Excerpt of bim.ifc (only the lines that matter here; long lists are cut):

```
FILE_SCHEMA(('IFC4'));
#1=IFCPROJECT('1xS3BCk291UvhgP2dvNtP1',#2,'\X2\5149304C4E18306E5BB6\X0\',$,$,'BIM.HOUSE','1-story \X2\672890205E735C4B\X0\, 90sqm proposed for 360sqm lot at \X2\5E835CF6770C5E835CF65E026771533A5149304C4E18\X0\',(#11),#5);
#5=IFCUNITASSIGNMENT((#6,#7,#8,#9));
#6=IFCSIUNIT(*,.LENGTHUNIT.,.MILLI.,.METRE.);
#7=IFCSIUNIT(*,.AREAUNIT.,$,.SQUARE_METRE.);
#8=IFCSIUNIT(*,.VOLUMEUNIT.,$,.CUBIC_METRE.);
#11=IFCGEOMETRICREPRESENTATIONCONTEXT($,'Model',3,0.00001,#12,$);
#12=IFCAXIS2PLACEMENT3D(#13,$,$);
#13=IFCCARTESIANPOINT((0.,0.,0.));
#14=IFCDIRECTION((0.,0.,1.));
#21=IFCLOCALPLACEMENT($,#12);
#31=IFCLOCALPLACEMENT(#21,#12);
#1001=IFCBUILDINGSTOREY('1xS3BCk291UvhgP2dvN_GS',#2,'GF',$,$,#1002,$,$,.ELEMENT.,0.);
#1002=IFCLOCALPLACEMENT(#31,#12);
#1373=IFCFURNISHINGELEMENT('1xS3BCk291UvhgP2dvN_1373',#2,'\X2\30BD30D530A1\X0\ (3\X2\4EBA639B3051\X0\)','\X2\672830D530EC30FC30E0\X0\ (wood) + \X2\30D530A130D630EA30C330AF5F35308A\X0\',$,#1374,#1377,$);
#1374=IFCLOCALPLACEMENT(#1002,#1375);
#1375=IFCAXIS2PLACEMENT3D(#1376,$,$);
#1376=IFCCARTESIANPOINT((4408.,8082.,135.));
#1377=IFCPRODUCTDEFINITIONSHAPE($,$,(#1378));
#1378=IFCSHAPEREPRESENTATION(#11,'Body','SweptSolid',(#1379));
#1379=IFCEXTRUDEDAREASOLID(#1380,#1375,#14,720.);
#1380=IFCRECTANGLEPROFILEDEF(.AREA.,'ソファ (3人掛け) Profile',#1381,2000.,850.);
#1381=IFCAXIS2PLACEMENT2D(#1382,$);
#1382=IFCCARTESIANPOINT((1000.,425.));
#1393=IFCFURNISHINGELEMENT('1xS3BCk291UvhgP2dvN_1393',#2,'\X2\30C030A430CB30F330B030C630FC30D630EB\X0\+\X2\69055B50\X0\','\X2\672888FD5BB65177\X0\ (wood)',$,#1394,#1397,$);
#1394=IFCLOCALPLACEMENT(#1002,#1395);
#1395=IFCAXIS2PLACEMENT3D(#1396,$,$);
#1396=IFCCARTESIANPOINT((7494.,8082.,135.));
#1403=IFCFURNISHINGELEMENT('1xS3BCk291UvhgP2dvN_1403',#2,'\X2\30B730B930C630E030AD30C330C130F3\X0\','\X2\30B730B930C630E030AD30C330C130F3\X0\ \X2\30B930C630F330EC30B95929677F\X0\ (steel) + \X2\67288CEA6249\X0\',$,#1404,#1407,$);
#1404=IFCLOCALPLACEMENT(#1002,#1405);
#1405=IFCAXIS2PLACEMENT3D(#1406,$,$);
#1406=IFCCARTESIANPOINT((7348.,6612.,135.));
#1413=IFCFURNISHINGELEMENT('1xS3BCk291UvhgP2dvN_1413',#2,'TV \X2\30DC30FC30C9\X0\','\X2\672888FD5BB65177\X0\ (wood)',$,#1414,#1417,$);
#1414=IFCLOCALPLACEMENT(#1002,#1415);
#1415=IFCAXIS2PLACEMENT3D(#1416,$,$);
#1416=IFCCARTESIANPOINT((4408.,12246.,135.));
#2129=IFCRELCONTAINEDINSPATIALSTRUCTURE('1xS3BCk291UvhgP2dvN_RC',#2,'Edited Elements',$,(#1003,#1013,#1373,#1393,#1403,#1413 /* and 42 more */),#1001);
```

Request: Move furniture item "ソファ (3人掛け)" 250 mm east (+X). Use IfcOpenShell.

```python
import ifcopenshell
import ifcopenshell.api.geometry
import ifcopenshell.util.placement
import ifcopenshell.util.unit

model = ifcopenshell.open("bim.ifc")
unit_scale = ifcopenshell.util.unit.calculate_unit_scale(model)

item = model.by_id(1373)
matrix = ifcopenshell.util.placement.get_local_placement(item.ObjectPlacement)
matrix[0, 3] += 0.25 / unit_scale
ifcopenshell.api.geometry.edit_object_placement(model, product=item, matrix=matrix, is_si=False)

print(ifcopenshell.util.placement.get_local_placement(item.ObjectPlacement).round(3) + 0.0)

model.write("bim-out.ifc")
```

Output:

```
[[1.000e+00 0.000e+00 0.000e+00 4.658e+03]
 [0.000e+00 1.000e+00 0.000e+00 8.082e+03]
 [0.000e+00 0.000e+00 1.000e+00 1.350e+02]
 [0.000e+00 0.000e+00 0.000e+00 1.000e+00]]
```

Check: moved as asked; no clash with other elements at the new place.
